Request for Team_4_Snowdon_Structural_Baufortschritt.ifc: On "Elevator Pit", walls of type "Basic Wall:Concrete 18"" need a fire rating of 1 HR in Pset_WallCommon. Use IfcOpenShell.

First a look at what the model holds.

```python
import ifcopenshell
import ifcopenshell.util.element

model = ifcopenshell.open("Team_4_Snowdon_Structural_Baufortschritt.ifc")
print(model.schema)
storey = next(s for s in model.by_type("IfcBuildingStorey") if s.Name == "Elevator Pit")
walls = [e for e in ifcopenshell.util.element.get_decomposition(storey) if e.is_a("IfcWall")]
seen = {}
for e in walls:
    element_type = ifcopenshell.util.element.get_type(e)
    key = (element_type.Name if element_type != e and element_type else None, ifcopenshell.util.element.get_pset(e, "Pset_WallCommon", "FireRating"))
    seen[key] = seen.get(key, 0) + 1
for (name, value), count in sorted(seen.items(), key=str):
    print(count, "x", name, "|", value)
```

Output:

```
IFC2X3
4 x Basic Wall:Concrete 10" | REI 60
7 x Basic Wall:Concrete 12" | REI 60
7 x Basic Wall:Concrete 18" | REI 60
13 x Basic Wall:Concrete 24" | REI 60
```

```python
import ifcopenshell
import ifcopenshell.api.pset
import ifcopenshell.util.element

model = ifcopenshell.open("Team_4_Snowdon_Structural_Baufortschritt.ifc")

storey = next(s for s in model.by_type("IfcBuildingStorey") if s.Name == "Elevator Pit")
walls = [e for e in ifcopenshell.util.element.get_decomposition(storey) if e.is_a("IfcWall")]

count = 0
for e in walls:
    element_type = ifcopenshell.util.element.get_type(e)
    if element_type in (None, e) or element_type.Name != 'Basic Wall:Concrete 18"':
        continue
    # add_pset returns the element's existing set when there is one.
    pset = ifcopenshell.api.pset.add_pset(model, product=e, name="Pset_WallCommon")
    ifcopenshell.api.pset.edit_pset(model, pset=pset, properties={"FireRating": "1 HR"})
    count += 1

print(count, "walls updated")

model.write("Team_4_Snowdon_Structural_Baufortschritt_edited.ifc")
```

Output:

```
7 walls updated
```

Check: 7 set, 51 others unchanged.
